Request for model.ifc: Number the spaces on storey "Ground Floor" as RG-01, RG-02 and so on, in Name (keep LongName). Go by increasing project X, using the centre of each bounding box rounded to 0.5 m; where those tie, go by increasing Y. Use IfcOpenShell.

First a look at what the model holds.

```python
import ifcopenshell
import ifcopenshell.util.element
import ifcopenshell.util.placement

model = ifcopenshell.open("model.ifc")
print(model.schema)
storey = next(s for s in model.by_type("IfcBuildingStorey") if s.Name == "Ground Floor")
spaces = [e for e in ifcopenshell.util.element.get_decomposition(storey) if e.is_a("IfcSpace")]
for e in sorted(spaces, key=lambda e: e.id()):
    origin = ifcopenshell.util.placement.get_local_placement(e.ObjectPlacement)[:3, 3]
    print(e.id(), e.Name, e.LongName, origin.round(2) + 0.0, sep=" | ")
```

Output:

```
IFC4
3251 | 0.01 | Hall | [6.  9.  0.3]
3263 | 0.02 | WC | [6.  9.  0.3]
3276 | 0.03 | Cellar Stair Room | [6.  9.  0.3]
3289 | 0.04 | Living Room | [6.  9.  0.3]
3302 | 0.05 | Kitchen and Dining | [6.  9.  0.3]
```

```python
import ifcopenshell
import ifcopenshell.geom
import ifcopenshell.util.element
import ifcopenshell.util.shape

model = ifcopenshell.open("model.ifc")
settings = ifcopenshell.geom.settings()
settings.set("use-world-coords", True)


def centre(element):
    shape = ifcopenshell.geom.create_shape(settings, element)
    return ifcopenshell.util.shape.get_bbox_centroid(shape.geometry)


storey = next(s for s in model.by_type("IfcBuildingStorey") if s.Name == "Ground Floor")
spaces = [e for e in ifcopenshell.util.element.get_decomposition(storey) if e.is_a("IfcSpace")]

# Insertion points can sit at a corner or the storey origin, so sort by the geometry (in metres).
centres = {e: centre(e) for e in spaces}
spaces.sort(key=lambda e: (round(centres[e][0] / 0.5), centres[e][1]))

for i, e in enumerate(spaces, start=1):
    number = f"RG-{i:02d}"
    e.Name = number
    print(e.id(), number)

model.write("model_edited.ifc")
```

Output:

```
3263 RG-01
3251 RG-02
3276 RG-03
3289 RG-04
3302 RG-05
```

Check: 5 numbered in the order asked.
